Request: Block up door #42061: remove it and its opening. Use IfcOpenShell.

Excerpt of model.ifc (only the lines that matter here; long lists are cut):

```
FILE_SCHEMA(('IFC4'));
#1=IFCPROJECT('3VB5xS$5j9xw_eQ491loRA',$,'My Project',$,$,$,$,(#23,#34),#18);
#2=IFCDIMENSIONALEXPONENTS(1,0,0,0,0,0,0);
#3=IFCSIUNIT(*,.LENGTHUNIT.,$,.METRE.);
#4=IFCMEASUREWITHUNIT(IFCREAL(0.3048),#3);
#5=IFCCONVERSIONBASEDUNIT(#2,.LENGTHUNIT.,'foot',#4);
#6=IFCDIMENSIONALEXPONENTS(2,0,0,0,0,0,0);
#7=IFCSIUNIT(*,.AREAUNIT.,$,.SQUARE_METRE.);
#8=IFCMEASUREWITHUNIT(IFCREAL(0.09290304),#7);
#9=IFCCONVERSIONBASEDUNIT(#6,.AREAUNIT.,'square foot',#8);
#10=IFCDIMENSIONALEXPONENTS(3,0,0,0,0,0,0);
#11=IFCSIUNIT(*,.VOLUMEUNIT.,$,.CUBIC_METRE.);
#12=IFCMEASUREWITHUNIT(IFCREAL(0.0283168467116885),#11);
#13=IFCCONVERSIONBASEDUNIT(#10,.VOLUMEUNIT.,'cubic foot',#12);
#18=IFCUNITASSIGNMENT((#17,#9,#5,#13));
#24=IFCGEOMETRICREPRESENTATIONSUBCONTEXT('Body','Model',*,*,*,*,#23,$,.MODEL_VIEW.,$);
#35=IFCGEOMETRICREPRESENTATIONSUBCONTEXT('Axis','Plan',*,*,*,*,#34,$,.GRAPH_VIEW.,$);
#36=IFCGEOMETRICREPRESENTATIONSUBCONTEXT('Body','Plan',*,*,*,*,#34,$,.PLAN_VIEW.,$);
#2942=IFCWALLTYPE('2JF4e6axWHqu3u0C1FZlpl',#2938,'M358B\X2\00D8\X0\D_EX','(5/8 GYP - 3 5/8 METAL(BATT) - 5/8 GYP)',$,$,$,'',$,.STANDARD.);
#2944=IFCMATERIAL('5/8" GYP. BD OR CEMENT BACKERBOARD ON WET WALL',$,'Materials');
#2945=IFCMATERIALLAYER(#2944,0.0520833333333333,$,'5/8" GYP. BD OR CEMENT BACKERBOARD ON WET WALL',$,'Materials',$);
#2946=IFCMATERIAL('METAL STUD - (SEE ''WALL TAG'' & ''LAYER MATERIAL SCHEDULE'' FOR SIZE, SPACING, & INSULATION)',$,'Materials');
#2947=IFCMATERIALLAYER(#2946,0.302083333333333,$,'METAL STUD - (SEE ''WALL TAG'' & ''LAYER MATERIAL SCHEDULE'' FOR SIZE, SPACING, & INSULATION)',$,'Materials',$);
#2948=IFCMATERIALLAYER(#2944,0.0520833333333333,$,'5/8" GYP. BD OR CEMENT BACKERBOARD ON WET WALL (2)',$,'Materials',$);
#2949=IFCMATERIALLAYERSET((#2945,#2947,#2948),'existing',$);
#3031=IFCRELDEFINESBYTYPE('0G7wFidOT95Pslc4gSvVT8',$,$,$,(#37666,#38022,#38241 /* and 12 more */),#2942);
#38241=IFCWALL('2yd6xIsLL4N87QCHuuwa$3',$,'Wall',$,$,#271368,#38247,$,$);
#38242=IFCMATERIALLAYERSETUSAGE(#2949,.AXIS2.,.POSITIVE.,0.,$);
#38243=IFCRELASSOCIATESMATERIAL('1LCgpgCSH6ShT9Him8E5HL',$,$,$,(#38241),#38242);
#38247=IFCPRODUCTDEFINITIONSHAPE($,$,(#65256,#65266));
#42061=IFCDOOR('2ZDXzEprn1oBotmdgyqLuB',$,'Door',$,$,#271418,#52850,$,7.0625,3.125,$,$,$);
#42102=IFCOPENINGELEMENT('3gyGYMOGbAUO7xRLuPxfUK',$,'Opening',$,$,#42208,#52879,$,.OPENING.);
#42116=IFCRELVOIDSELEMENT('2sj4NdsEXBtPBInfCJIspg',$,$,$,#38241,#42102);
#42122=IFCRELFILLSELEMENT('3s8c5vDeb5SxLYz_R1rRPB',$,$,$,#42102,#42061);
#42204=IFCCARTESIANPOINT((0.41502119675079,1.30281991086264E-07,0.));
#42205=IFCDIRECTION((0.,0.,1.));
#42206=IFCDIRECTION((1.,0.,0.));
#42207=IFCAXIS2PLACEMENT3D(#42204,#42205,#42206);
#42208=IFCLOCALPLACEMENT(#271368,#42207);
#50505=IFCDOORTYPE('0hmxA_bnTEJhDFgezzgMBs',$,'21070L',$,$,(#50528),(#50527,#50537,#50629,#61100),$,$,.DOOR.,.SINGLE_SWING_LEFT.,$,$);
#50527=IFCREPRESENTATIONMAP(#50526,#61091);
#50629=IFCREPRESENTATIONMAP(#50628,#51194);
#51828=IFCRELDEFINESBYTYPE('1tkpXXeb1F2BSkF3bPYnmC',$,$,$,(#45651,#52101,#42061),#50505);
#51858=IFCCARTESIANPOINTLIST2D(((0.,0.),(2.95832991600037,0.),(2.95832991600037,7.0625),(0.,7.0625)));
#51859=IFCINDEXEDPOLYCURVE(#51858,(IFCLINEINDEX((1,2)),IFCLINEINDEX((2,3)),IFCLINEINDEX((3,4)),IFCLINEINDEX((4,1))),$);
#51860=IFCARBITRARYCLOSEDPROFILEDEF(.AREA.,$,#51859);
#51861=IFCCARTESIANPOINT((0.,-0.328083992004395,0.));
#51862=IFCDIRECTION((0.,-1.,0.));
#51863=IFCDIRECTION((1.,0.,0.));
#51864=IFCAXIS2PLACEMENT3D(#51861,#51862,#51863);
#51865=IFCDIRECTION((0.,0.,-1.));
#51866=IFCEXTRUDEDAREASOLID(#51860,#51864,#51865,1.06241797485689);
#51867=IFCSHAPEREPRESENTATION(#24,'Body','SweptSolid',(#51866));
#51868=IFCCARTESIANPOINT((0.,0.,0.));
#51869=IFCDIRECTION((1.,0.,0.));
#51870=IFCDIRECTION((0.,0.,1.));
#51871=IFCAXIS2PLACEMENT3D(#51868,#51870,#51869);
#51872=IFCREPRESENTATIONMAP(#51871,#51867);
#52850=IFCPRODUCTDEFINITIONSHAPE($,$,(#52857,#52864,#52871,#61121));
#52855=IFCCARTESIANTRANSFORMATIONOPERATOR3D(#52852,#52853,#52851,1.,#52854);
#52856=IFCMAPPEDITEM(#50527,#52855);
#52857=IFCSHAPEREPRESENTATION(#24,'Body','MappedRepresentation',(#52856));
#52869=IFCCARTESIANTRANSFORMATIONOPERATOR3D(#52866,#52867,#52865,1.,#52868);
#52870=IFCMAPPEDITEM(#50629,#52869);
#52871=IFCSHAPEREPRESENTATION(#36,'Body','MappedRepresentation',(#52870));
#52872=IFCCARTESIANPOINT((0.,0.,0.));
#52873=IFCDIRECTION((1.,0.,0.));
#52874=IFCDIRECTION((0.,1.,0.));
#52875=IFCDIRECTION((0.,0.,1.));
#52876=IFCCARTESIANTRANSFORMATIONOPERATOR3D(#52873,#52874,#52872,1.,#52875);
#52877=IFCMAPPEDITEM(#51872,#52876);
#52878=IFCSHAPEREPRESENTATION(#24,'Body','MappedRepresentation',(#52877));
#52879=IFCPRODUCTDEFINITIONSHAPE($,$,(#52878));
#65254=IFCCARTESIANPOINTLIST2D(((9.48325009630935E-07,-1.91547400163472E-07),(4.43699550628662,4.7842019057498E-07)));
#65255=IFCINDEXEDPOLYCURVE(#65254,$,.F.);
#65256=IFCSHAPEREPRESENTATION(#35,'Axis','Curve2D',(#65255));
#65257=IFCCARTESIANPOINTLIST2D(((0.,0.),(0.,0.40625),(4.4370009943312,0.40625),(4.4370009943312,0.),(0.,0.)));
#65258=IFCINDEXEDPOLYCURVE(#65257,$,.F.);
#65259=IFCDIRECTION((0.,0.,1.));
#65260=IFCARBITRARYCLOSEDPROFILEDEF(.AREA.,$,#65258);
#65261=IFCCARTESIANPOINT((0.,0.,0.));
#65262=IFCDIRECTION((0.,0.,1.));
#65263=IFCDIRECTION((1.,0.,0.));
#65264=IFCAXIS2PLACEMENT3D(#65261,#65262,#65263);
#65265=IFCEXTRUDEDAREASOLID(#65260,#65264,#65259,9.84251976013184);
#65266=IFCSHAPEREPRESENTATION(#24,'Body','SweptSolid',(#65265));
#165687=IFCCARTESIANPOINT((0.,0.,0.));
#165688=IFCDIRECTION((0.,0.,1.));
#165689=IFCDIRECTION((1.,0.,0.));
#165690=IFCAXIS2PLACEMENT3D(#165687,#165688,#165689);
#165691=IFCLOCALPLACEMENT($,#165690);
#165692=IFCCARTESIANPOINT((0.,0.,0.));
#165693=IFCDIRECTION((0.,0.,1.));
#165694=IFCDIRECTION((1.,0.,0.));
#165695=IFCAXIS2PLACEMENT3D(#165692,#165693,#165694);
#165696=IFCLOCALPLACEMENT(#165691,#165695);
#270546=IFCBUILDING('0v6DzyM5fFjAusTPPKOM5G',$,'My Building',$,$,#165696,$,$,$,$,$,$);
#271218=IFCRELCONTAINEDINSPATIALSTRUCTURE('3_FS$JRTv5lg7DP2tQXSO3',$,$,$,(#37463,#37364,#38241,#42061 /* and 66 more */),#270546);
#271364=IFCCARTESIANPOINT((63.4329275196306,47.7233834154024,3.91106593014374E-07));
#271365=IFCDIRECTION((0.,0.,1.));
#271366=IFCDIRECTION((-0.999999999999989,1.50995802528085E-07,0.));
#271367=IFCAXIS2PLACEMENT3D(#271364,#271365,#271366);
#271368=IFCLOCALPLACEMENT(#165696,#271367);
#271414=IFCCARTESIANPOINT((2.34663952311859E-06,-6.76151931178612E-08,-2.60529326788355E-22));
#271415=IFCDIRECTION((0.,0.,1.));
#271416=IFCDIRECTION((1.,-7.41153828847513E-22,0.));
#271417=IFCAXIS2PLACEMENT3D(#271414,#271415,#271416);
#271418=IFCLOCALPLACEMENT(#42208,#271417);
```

```python
import ifcopenshell
import ifcopenshell.api.feature
import ifcopenshell.api.root
import ifcopenshell.geom
import ifcopenshell.util.shape

model = ifcopenshell.open("model.ifc")
settings = ifcopenshell.geom.settings()


def volume(element):
    """Net volume in cubic metres, openings subtracted."""
    shape = ifcopenshell.geom.create_shape(settings, element)
    return ifcopenshell.util.shape.get_volume(shape.geometry)


door = model.by_guid("2ZDXzEprn1oBotmdgyqLuB")
opening = door.FillsVoids[0].RelatingOpeningElement
wall = opening.VoidsElements[0].RelatingBuildingElement
before = volume(wall)

ifcopenshell.api.root.remove_product(model, product=door)
ifcopenshell.api.feature.remove_feature(model, feature=opening)

after = volume(wall)

print(f"wall volume {before:.3f} -> {after:.3f} m3")

model.write("model_edited.ifc")
```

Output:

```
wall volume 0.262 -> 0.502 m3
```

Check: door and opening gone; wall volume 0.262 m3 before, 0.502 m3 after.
